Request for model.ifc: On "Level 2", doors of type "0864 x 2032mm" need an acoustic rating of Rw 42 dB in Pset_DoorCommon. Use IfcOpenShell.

First a look at what the model holds.

```python
import ifcopenshell
import ifcopenshell.util.element

model = ifcopenshell.open("model.ifc")
print(model.schema)
storey = next(s for s in model.by_type("IfcBuildingStorey") if s.Name == "Level 2")
doors = [e for e in ifcopenshell.util.element.get_decomposition(storey) if e.is_a("IfcDoor")]
seen = {}
for e in doors:
    element_type = ifcopenshell.util.element.get_type(e)
    key = (element_type.Name if element_type != e and element_type else None, ifcopenshell.util.element.get_pset(e, "Pset_DoorCommon", "AcousticRating"))
    seen[key] = seen.get(key, 0) + 1
for (name, value), count in sorted(seen.items(), key=str):
    print(count, "x", name, "|", value)
```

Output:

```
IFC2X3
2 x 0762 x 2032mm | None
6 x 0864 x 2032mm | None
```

```python
import ifcopenshell
import ifcopenshell.api.pset
import ifcopenshell.util.element

model = ifcopenshell.open("model.ifc")

storey = next(s for s in model.by_type("IfcBuildingStorey") if s.Name == "Level 2")
doors = [e for e in ifcopenshell.util.element.get_decomposition(storey) if e.is_a("IfcDoor")]

count = 0
for e in doors:
    element_type = ifcopenshell.util.element.get_type(e)
    if element_type in (None, e) or element_type.Name != "0864 x 2032mm":
        continue
    # add_pset returns the element's existing set when there is one.
    pset = ifcopenshell.api.pset.add_pset(model, product=e, name="Pset_DoorCommon")
    ifcopenshell.api.pset.edit_pset(model, pset=pset, properties={"AcousticRating": "Rw 42 dB"})
    count += 1

print(count, "doors updated")

model.write("model_v2.ifc")
```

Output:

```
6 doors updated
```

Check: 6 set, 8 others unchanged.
